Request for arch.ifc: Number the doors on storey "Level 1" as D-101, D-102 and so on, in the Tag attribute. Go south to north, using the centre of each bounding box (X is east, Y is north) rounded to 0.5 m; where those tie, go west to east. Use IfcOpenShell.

First a look at what the model holds.

```python
import ifcopenshell
import ifcopenshell.util.element
import ifcopenshell.util.placement

model = ifcopenshell.open("arch.ifc")
print(model.schema)
storey = next(s for s in model.by_type("IfcBuildingStorey") if s.Name == "Level 1")
doors = [e for e in ifcopenshell.util.element.get_decomposition(storey) if e.is_a("IfcDoor")]
for e in sorted(doors, key=lambda e: e.id()):
    origin = ifcopenshell.util.placement.get_local_placement(e.ObjectPlacement)[:3, 3]
    print(e.id(), e.Tag, e.Name, origin.round(2) + 0.0, sep=" | ")
```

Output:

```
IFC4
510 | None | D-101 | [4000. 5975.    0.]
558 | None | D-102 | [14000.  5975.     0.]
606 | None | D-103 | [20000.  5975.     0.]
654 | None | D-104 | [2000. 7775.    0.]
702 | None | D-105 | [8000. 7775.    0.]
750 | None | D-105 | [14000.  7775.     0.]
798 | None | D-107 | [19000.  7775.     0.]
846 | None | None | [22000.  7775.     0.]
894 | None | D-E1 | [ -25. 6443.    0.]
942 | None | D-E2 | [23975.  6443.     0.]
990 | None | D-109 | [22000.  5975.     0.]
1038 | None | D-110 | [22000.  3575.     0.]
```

```python
import ifcopenshell
import ifcopenshell.geom
import ifcopenshell.util.element
import ifcopenshell.util.shape

model = ifcopenshell.open("arch.ifc")
settings = ifcopenshell.geom.settings()
settings.set("use-world-coords", True)


def centre(element):
    shape = ifcopenshell.geom.create_shape(settings, element)
    return ifcopenshell.util.shape.get_bbox_centroid(shape.geometry)


storey = next(s for s in model.by_type("IfcBuildingStorey") if s.Name == "Level 1")
doors = [e for e in ifcopenshell.util.element.get_decomposition(storey) if e.is_a("IfcDoor")]

# Insertion points can sit at a corner or the storey origin, so sort by the geometry (in metres).
centres = {e: centre(e) for e in doors}
doors.sort(key=lambda e: (round(centres[e][1] / 0.5), centres[e][0]))

for i, e in enumerate(doors, start=1):
    number = f"D-1{i:02d}"
    e.Tag = number
    print(e.id(), number)

model.write("arch-out.ifc")
```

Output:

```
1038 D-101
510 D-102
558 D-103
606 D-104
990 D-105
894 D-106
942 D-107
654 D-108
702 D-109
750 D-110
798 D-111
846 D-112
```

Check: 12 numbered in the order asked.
